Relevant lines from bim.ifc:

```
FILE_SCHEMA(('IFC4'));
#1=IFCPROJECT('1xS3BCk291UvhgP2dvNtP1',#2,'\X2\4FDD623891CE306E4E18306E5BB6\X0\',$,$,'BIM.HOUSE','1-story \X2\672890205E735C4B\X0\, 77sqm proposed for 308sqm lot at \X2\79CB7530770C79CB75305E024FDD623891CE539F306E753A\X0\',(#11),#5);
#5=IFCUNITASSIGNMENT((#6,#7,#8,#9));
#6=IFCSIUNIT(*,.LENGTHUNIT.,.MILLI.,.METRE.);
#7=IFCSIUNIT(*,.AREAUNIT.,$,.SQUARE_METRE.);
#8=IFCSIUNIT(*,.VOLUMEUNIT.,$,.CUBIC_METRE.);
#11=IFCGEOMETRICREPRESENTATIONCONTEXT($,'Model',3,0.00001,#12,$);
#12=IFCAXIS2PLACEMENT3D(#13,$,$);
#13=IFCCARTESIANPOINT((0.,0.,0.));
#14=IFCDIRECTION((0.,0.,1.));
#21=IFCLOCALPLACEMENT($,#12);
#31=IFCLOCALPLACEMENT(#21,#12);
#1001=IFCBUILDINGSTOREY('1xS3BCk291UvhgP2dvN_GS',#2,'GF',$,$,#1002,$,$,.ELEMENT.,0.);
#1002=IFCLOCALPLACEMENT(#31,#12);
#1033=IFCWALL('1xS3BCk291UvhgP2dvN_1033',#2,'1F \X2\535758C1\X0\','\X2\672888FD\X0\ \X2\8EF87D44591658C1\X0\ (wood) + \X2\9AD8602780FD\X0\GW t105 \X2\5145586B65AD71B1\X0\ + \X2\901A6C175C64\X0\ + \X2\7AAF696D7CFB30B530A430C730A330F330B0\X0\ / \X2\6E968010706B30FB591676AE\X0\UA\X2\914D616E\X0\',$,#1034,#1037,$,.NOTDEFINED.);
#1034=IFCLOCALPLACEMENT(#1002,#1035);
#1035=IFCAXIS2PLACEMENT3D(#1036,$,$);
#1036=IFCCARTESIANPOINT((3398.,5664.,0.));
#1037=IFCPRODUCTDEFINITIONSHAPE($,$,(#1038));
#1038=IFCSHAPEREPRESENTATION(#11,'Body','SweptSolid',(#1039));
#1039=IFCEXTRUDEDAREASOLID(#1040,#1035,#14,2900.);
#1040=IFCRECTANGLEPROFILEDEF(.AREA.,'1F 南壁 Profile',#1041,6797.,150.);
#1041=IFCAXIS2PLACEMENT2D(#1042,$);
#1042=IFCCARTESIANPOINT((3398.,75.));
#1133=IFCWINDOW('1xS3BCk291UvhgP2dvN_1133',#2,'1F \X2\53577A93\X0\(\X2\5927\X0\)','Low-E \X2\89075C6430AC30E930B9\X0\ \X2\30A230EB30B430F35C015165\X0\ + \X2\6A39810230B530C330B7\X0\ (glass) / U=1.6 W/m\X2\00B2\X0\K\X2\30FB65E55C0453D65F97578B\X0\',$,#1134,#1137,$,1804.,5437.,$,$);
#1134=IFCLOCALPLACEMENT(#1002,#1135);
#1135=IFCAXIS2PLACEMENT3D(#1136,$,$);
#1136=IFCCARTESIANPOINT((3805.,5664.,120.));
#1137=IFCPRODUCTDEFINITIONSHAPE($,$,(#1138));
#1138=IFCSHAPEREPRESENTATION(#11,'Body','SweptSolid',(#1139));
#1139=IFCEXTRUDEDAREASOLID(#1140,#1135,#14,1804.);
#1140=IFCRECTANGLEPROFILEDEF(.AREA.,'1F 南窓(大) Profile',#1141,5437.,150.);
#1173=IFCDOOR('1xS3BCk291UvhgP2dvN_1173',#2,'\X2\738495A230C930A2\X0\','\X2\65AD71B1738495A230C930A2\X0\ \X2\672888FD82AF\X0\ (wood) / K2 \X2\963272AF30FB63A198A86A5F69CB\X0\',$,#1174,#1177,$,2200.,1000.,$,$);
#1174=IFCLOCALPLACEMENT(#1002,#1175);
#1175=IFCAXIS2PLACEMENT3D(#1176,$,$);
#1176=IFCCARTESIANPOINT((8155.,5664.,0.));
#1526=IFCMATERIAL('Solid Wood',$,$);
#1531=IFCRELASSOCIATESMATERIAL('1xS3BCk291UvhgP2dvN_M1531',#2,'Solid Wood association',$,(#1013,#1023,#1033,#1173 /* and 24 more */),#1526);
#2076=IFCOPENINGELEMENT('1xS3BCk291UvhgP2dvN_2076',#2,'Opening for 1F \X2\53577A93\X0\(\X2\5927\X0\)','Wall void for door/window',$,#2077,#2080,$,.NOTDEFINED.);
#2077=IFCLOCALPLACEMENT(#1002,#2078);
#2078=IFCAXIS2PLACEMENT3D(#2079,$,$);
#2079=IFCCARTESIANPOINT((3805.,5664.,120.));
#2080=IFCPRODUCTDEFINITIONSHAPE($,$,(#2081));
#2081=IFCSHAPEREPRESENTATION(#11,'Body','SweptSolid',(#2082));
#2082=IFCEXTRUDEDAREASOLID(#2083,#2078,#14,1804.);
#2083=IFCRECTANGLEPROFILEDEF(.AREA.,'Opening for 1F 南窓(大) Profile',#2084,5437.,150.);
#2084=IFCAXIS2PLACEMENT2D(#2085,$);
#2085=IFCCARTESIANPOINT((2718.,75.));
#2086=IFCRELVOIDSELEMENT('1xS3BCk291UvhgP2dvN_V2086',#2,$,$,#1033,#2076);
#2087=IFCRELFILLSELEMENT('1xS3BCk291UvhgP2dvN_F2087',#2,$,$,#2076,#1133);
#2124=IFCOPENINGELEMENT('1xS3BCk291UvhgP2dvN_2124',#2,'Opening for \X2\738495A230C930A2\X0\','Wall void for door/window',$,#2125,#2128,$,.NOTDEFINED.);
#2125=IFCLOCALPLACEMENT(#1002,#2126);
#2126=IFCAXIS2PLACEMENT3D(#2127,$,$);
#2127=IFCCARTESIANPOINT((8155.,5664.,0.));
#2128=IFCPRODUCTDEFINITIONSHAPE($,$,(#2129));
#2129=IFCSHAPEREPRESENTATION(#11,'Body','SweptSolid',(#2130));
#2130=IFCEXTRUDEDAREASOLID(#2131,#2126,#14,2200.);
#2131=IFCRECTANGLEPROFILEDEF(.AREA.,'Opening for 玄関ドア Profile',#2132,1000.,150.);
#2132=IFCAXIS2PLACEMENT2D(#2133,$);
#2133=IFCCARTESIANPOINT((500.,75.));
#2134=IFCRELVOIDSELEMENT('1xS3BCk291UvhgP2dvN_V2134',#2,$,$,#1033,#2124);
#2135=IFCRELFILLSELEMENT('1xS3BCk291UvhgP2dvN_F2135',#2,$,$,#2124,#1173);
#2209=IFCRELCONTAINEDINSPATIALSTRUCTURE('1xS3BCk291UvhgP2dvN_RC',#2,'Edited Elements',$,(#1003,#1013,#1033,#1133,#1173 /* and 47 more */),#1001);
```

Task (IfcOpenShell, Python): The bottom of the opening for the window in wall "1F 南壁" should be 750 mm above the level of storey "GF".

```python
import numpy as np
import ifcopenshell
import ifcopenshell.api.geometry
import ifcopenshell.geom
import ifcopenshell.util.element
import ifcopenshell.util.placement
import ifcopenshell.util.shape
import ifcopenshell.util.unit

model = ifcopenshell.open("bim.ifc")
unit_scale = ifcopenshell.util.unit.calculate_unit_scale(model)

window = model.by_id(1133)
opening = window.FillsVoids[0].RelatingOpeningElement
storey = ifcopenshell.util.element.get_container(window, ifc_class="IfcBuildingStorey")
level = ifcopenshell.util.placement.get_local_placement(storey.ObjectPlacement)[2, 3]

# The opening's origin need not be at the sill, so measure its lowest point.
shape = ifcopenshell.geom.create_shape(ifcopenshell.geom.settings(), opening)
bottom = ifcopenshell.util.shape.get_shape_bottom_elevation(shape, shape.geometry) / unit_scale
dz = level + 750.0 - bottom

shift = np.array([0.0, 0.0, dz])
# The window is not placed relative to its opening, so move both.
for product in (opening, window):
    matrix = ifcopenshell.util.placement.get_local_placement(product.ObjectPlacement)
    matrix[:3, 3] += shift
    ifcopenshell.api.geometry.edit_object_placement(model, product=product, matrix=matrix, is_si=False)

print(f"moved by {dz * unit_scale:+.3f} m")

model.write("bim_updated.ifc")
```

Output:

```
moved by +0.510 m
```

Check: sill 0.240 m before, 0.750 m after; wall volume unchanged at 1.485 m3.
